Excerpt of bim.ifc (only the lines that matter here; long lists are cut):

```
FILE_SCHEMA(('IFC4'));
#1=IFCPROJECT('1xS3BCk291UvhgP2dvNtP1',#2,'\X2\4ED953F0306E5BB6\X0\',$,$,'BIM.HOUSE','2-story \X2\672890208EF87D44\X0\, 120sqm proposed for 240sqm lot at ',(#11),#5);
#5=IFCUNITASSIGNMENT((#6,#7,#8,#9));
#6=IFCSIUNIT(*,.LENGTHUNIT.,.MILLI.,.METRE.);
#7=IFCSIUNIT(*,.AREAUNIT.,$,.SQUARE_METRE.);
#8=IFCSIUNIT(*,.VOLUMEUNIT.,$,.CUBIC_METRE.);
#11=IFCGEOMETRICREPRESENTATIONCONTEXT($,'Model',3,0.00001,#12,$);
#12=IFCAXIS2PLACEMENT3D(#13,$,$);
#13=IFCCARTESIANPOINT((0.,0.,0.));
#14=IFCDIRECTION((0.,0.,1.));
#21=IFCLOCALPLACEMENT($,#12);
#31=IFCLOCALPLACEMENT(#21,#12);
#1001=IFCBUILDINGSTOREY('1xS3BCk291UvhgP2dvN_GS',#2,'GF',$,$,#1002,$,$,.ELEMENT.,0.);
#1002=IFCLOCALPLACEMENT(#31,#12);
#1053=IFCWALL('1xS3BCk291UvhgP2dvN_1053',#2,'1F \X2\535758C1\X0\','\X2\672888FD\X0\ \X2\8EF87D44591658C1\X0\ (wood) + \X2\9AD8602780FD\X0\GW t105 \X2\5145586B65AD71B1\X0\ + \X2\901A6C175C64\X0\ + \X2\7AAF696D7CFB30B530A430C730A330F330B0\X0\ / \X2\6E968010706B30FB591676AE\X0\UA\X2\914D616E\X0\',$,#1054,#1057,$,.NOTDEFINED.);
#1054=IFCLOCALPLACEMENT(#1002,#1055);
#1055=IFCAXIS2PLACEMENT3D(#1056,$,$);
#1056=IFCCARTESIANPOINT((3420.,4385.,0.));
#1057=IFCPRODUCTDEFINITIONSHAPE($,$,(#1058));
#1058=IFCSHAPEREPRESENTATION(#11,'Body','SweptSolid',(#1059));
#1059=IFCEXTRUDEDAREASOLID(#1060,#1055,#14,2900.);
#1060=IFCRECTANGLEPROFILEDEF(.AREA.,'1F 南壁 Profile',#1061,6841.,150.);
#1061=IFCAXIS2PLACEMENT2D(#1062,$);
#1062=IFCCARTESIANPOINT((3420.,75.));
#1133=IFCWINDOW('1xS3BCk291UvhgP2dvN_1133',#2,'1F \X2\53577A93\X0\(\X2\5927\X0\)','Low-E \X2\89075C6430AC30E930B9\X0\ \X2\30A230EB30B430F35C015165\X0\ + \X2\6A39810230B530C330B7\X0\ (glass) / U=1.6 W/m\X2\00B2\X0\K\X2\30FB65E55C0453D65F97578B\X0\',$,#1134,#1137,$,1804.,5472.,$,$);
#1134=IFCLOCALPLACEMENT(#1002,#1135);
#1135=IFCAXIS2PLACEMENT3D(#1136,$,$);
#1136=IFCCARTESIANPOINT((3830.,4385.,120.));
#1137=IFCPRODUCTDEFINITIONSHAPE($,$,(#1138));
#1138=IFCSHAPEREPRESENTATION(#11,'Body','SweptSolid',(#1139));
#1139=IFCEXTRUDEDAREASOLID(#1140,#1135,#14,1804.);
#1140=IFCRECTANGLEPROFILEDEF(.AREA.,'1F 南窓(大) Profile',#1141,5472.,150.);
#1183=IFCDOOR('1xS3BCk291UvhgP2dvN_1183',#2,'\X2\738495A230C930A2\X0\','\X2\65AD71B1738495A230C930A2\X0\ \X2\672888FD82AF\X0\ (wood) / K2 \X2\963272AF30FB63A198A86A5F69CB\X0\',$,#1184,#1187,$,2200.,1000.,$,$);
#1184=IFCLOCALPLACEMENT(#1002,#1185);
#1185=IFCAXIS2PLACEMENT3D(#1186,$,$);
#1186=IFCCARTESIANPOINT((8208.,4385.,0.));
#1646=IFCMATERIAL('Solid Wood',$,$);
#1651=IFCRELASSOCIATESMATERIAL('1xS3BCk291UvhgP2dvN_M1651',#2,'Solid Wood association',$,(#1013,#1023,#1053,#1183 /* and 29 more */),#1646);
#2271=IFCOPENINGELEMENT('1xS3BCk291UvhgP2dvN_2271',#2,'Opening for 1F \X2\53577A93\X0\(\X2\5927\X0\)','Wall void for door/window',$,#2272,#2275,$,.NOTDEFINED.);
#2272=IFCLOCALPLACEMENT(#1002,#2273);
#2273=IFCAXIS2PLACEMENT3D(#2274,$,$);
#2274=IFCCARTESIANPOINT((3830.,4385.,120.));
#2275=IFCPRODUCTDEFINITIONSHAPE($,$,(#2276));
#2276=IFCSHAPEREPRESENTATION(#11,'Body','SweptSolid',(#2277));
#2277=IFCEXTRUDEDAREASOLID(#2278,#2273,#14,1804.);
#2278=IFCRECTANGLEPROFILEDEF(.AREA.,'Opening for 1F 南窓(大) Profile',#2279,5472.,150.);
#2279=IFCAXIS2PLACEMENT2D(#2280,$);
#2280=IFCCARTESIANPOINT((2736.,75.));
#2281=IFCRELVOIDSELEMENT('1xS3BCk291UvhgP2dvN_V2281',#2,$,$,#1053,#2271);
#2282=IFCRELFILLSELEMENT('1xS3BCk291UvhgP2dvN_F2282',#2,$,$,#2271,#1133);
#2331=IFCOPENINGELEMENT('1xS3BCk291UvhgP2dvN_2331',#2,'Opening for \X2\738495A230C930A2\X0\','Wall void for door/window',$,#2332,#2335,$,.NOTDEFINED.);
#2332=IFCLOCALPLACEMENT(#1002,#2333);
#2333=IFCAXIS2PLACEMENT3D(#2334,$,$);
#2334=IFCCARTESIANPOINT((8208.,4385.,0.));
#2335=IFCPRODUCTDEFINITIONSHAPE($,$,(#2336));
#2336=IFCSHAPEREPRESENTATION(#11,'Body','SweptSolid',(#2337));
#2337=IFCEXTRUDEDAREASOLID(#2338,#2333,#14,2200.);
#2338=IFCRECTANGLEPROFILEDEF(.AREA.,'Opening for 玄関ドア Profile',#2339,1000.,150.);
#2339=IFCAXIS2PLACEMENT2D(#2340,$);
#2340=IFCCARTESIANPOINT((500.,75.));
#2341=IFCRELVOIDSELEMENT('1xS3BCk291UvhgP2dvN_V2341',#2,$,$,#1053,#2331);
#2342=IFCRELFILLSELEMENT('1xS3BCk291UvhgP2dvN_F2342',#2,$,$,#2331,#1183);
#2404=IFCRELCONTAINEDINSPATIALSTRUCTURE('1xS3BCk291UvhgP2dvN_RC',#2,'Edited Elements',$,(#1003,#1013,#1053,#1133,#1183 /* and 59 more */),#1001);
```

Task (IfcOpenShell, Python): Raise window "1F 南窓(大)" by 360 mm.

```python
import numpy as np
import ifcopenshell
import ifcopenshell.api.geometry
import ifcopenshell.util.placement
import ifcopenshell.util.unit

model = ifcopenshell.open("bim.ifc")
unit_scale = ifcopenshell.util.unit.calculate_unit_scale(model)

window = model.by_guid("1xS3BCk291UvhgP2dvN_1133")
opening = window.FillsVoids[0].RelatingOpeningElement
dz = 0.36 / unit_scale

shift = np.array([0.0, 0.0, dz])
# The window is not placed relative to its opening, so move both.
for product in (opening, window):
    matrix = ifcopenshell.util.placement.get_local_placement(product.ObjectPlacement)
    matrix[:3, 3] += shift
    ifcopenshell.api.geometry.edit_object_placement(model, product=product, matrix=matrix, is_si=False)

print(f"moved by {dz * unit_scale:+.3f} m")

model.write("bim_v2.ifc")
```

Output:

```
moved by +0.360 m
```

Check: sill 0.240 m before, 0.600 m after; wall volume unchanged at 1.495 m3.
